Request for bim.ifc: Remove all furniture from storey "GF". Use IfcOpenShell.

First a look at what the model holds.

```python
import ifcopenshell
import ifcopenshell.util.element

model = ifcopenshell.open("bim.ifc")
print(model.schema)
storey = next(s for s in model.by_type("IfcBuildingStorey") if s.Name == "GF")
furniture = [e for e in ifcopenshell.util.element.get_decomposition(storey) if e.is_a("IfcFurnishingElement")]
seen = {}
for e in furniture:
    element_type = ifcopenshell.util.element.get_type(e)
    name = element_type.Name if element_type not in (None, e) else None
    seen[name] = seen.get(name, 0) + 1
for name, count in sorted(seen.items(), key=str):
    print(count, "x", name)
```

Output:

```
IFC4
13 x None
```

```python
import ifcopenshell
import ifcopenshell.api.root
import ifcopenshell.util.element

model = ifcopenshell.open("bim.ifc")

storey = next(s for s in model.by_type("IfcBuildingStorey") if s.Name == "GF")
furniture = [e for e in ifcopenshell.util.element.get_decomposition(storey) if e.is_a("IfcFurnishingElement")]

for e in furniture:
    ifcopenshell.api.root.remove_product(model, product=e)
print(len(furniture), "removed")

model.write("bim_v2.ifc")
```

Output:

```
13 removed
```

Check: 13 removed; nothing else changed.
